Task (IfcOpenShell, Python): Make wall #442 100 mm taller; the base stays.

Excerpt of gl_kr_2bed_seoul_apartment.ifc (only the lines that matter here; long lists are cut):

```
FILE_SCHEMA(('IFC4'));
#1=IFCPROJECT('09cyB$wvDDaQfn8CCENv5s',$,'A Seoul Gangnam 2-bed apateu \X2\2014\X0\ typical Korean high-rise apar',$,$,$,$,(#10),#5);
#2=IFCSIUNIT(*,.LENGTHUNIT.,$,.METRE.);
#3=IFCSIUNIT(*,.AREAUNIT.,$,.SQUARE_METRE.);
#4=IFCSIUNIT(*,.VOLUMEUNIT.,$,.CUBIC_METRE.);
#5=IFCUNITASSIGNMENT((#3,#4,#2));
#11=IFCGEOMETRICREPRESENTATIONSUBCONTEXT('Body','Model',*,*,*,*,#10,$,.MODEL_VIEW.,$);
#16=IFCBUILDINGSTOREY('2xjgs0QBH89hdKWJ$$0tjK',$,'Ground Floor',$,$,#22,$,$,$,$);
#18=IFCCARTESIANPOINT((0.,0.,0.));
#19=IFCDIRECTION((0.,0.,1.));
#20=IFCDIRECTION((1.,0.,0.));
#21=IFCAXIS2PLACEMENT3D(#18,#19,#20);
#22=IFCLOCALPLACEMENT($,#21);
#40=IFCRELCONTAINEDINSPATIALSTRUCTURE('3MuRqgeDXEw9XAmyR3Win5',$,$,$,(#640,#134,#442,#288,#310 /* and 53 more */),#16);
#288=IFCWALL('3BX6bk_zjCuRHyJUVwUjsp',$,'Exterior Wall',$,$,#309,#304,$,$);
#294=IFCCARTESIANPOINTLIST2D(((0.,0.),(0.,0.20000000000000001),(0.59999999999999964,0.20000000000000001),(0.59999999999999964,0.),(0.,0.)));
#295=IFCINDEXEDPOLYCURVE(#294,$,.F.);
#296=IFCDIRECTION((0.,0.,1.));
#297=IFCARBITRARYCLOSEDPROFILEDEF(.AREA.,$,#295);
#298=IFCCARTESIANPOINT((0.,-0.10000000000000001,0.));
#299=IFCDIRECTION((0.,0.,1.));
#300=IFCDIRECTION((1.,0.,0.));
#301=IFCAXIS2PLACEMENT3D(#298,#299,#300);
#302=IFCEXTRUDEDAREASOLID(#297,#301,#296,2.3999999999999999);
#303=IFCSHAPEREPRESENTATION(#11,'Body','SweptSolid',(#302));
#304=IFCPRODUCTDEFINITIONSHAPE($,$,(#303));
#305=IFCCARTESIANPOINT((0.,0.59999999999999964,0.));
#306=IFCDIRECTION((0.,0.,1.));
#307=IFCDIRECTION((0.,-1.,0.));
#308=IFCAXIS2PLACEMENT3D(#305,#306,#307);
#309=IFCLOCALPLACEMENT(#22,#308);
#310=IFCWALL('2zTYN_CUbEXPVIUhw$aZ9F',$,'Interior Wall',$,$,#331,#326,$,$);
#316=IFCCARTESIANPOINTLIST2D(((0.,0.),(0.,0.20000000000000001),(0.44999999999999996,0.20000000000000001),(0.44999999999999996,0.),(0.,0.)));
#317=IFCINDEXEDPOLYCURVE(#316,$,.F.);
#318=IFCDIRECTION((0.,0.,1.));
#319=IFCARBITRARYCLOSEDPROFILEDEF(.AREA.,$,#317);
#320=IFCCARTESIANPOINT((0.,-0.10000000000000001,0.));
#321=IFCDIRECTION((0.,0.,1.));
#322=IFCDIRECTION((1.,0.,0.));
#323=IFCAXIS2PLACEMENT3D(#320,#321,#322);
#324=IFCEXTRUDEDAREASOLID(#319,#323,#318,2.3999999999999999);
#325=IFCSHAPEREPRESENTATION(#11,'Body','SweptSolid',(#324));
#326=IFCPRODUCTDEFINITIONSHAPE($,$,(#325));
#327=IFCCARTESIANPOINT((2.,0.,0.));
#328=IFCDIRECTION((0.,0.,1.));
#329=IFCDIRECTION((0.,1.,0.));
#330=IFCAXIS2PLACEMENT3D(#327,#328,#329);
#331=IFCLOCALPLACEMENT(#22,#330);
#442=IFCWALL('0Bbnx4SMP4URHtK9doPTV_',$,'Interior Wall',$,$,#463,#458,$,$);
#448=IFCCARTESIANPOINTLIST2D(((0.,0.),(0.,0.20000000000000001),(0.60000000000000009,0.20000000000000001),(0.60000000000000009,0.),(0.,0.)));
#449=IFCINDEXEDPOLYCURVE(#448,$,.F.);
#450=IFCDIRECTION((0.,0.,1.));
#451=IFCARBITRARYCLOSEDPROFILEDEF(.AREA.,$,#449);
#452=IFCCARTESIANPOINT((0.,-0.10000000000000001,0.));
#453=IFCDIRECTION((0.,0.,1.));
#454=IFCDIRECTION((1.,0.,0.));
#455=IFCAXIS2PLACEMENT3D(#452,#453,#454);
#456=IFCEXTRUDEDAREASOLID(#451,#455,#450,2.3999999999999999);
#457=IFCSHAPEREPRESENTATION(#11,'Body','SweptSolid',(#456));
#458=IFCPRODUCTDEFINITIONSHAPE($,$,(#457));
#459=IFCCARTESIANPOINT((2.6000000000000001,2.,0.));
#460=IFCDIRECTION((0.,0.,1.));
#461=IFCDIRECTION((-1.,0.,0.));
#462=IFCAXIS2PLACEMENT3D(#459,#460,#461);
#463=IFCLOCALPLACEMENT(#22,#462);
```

```python
import ifcopenshell
import ifcopenshell.geom
import ifcopenshell.util.representation
import ifcopenshell.util.shape
import ifcopenshell.util.unit

model = ifcopenshell.open("gl_kr_2bed_seoul_apartment.ifc")
unit_scale = ifcopenshell.util.unit.calculate_unit_scale(model)
settings = ifcopenshell.geom.settings()


def volume(element):
    """Net volume in cubic metres, openings subtracted."""
    shape = ifcopenshell.geom.create_shape(settings, element)
    return ifcopenshell.util.shape.get_volume(shape.geometry)


wall = model.by_id(442)
before = volume(wall)

body = ifcopenshell.util.representation.get_representation(wall, "Model", "Body")
solid = body.Items[0]
old_height = solid.Depth
solid.Depth += 0.1 / unit_scale
after = volume(wall)

print(f"height {old_height:g} -> {solid.Depth:g}, volume {before:.3f} -> {after:.3f} m3")

model.write("gl_kr_2bed_seoul_apartment_rev.ifc")
```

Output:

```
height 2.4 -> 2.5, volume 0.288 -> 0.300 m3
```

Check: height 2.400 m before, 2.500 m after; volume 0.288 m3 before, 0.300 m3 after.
